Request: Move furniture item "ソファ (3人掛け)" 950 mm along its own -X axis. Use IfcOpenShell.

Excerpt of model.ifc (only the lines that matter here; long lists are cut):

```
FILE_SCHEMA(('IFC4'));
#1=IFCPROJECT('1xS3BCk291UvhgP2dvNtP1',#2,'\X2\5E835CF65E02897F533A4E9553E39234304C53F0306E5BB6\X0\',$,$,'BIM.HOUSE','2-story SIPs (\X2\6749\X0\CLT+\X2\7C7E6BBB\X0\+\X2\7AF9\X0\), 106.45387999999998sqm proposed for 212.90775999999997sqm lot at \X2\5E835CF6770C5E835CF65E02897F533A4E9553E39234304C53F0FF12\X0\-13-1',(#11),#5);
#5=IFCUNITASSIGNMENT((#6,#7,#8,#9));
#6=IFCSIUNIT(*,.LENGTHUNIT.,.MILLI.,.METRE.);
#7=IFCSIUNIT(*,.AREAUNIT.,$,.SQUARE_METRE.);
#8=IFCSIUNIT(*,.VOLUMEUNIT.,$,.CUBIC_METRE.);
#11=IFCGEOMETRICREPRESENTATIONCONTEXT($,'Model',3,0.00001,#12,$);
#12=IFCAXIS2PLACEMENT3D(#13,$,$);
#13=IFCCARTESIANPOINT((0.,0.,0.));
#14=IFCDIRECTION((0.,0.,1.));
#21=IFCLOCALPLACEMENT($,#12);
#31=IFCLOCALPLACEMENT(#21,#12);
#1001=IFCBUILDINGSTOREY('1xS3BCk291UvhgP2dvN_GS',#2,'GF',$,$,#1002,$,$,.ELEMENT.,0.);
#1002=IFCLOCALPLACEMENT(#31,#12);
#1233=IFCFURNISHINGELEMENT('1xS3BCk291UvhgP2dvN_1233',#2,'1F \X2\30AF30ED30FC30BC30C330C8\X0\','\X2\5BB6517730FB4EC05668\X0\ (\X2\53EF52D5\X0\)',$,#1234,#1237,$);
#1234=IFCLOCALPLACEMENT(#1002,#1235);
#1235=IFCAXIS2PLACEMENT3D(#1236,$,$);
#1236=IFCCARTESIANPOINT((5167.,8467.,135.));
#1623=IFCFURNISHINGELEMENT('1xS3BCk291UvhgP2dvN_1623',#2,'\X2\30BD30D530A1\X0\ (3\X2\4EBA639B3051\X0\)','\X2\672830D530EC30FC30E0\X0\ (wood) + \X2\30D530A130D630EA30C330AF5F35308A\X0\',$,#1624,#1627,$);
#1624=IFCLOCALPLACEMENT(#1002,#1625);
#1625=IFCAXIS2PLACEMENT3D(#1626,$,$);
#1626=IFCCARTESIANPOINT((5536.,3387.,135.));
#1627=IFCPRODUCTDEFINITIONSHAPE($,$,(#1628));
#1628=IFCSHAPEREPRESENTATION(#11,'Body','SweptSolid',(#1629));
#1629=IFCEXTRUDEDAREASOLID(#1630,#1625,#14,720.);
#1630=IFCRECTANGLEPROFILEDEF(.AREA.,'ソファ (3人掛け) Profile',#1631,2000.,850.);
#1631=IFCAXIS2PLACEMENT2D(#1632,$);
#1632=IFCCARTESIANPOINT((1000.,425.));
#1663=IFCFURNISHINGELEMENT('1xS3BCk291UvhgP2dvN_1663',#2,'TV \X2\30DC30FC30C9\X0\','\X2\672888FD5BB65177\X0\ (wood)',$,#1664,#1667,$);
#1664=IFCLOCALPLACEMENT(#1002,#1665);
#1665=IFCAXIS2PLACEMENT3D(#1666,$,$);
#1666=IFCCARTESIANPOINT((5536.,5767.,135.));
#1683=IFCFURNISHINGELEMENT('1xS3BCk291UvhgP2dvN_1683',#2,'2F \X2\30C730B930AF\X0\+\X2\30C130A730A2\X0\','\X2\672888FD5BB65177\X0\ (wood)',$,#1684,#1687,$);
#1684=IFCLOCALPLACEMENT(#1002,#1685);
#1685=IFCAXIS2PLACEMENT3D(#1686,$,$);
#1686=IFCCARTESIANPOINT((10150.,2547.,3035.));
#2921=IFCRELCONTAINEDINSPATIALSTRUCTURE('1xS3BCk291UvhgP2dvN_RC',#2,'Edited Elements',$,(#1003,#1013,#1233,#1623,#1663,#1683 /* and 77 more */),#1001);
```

```python
import ifcopenshell
import ifcopenshell.api.geometry
import ifcopenshell.util.placement
import ifcopenshell.util.unit

model = ifcopenshell.open("model.ifc")
unit_scale = ifcopenshell.util.unit.calculate_unit_scale(model)

item = model.by_id(1623)
matrix = ifcopenshell.util.placement.get_local_placement(item.ObjectPlacement)
matrix[:3, 3] -= matrix[:3, 0] * 0.95 / unit_scale
ifcopenshell.api.geometry.edit_object_placement(model, product=item, matrix=matrix, is_si=False)

print(ifcopenshell.util.placement.get_local_placement(item.ObjectPlacement).round(3) + 0.0)

model.write("model-out.ifc")
```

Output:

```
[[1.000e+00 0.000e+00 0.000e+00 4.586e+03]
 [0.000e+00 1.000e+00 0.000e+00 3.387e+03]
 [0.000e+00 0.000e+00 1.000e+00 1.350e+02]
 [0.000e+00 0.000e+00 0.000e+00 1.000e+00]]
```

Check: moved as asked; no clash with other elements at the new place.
